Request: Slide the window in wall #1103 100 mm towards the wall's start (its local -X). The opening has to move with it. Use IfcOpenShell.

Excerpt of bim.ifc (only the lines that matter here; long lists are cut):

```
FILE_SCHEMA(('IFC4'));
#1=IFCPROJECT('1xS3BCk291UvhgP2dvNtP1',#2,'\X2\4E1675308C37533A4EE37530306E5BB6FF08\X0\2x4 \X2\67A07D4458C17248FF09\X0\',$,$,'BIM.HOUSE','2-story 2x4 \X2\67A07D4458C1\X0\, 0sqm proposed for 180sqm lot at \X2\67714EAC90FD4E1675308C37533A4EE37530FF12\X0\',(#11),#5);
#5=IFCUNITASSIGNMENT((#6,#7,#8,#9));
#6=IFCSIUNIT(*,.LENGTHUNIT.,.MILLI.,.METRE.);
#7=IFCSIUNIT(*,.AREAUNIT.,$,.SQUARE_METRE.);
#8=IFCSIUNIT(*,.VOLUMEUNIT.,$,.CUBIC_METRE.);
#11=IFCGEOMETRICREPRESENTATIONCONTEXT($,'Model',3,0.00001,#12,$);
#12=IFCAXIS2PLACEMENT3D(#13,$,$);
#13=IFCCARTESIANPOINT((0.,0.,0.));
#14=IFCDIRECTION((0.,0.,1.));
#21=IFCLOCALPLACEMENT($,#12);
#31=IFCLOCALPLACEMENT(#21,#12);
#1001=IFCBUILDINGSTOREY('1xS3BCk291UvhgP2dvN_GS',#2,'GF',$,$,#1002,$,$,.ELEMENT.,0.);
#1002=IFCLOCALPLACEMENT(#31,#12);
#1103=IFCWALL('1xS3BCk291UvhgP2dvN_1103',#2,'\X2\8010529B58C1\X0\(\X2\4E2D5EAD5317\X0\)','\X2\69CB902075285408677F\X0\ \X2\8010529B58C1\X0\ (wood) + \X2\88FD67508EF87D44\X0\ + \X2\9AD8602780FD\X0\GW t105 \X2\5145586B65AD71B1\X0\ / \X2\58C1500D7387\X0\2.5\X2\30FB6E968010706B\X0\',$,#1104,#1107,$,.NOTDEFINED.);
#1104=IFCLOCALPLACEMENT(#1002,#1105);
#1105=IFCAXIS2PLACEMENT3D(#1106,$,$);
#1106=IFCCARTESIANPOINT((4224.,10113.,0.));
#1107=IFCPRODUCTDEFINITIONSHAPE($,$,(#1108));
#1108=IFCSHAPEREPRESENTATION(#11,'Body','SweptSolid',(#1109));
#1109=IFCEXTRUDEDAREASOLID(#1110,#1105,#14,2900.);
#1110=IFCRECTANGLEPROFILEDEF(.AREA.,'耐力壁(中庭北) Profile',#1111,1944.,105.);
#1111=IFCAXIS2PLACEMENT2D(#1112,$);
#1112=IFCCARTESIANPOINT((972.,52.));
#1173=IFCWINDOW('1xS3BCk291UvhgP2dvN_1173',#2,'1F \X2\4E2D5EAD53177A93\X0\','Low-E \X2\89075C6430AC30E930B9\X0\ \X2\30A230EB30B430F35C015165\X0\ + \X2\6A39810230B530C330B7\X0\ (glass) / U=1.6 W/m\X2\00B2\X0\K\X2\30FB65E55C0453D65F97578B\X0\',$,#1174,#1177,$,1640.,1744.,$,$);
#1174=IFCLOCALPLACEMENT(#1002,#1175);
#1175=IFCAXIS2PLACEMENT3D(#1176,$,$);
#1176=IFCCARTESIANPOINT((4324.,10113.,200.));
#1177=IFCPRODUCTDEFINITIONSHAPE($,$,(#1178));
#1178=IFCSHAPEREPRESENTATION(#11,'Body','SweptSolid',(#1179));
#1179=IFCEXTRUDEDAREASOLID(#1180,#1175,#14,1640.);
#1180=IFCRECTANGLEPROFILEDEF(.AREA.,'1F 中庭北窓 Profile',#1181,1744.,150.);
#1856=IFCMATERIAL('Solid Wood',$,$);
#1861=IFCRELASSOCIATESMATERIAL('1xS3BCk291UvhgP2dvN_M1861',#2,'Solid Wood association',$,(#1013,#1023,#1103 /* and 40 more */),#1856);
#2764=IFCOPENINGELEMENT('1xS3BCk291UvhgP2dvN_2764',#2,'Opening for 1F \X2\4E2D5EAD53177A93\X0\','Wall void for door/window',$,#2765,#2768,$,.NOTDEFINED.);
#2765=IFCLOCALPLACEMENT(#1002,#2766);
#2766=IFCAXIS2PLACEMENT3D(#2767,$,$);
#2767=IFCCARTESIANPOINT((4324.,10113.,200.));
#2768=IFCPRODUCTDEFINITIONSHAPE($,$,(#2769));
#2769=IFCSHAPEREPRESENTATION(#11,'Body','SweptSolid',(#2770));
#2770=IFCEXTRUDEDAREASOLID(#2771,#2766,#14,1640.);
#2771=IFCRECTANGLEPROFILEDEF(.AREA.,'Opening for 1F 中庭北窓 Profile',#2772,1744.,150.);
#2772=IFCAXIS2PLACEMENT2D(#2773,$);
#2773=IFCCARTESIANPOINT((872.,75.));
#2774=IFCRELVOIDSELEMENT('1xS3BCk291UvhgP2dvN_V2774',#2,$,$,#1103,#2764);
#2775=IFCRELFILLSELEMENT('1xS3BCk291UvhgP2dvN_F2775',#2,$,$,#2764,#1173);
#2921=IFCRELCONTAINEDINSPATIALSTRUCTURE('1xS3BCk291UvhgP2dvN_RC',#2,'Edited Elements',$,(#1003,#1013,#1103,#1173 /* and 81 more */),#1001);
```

```python
import ifcopenshell
import ifcopenshell.api.geometry
import ifcopenshell.util.placement
import ifcopenshell.util.unit

model = ifcopenshell.open("bim.ifc")
unit_scale = ifcopenshell.util.unit.calculate_unit_scale(model)

window = model.by_guid("1xS3BCk291UvhgP2dvN_1173")
opening = window.FillsVoids[0].RelatingOpeningElement
wall = opening.VoidsElements[0].RelatingBuildingElement

wall_matrix = ifcopenshell.util.placement.get_local_placement(wall.ObjectPlacement)
shift = wall_matrix[:3, 0] * -0.1 / unit_scale
before = ifcopenshell.util.placement.get_local_placement(window.ObjectPlacement)[:3, 3].copy()

# The window is not placed relative to its opening, so move both.
for product in (opening, window):
    matrix = ifcopenshell.util.placement.get_local_placement(product.ObjectPlacement)
    matrix[:3, 3] += shift
    ifcopenshell.api.geometry.edit_object_placement(model, product=product, matrix=matrix, is_si=False)

after = ifcopenshell.util.placement.get_local_placement(window.ObjectPlacement)[:3, 3]
print("window moved by", (after - before).round(3) + 0.0)

model.write("bim_v2.ifc")
```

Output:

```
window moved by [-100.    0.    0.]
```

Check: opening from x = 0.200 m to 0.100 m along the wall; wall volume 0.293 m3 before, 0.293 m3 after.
